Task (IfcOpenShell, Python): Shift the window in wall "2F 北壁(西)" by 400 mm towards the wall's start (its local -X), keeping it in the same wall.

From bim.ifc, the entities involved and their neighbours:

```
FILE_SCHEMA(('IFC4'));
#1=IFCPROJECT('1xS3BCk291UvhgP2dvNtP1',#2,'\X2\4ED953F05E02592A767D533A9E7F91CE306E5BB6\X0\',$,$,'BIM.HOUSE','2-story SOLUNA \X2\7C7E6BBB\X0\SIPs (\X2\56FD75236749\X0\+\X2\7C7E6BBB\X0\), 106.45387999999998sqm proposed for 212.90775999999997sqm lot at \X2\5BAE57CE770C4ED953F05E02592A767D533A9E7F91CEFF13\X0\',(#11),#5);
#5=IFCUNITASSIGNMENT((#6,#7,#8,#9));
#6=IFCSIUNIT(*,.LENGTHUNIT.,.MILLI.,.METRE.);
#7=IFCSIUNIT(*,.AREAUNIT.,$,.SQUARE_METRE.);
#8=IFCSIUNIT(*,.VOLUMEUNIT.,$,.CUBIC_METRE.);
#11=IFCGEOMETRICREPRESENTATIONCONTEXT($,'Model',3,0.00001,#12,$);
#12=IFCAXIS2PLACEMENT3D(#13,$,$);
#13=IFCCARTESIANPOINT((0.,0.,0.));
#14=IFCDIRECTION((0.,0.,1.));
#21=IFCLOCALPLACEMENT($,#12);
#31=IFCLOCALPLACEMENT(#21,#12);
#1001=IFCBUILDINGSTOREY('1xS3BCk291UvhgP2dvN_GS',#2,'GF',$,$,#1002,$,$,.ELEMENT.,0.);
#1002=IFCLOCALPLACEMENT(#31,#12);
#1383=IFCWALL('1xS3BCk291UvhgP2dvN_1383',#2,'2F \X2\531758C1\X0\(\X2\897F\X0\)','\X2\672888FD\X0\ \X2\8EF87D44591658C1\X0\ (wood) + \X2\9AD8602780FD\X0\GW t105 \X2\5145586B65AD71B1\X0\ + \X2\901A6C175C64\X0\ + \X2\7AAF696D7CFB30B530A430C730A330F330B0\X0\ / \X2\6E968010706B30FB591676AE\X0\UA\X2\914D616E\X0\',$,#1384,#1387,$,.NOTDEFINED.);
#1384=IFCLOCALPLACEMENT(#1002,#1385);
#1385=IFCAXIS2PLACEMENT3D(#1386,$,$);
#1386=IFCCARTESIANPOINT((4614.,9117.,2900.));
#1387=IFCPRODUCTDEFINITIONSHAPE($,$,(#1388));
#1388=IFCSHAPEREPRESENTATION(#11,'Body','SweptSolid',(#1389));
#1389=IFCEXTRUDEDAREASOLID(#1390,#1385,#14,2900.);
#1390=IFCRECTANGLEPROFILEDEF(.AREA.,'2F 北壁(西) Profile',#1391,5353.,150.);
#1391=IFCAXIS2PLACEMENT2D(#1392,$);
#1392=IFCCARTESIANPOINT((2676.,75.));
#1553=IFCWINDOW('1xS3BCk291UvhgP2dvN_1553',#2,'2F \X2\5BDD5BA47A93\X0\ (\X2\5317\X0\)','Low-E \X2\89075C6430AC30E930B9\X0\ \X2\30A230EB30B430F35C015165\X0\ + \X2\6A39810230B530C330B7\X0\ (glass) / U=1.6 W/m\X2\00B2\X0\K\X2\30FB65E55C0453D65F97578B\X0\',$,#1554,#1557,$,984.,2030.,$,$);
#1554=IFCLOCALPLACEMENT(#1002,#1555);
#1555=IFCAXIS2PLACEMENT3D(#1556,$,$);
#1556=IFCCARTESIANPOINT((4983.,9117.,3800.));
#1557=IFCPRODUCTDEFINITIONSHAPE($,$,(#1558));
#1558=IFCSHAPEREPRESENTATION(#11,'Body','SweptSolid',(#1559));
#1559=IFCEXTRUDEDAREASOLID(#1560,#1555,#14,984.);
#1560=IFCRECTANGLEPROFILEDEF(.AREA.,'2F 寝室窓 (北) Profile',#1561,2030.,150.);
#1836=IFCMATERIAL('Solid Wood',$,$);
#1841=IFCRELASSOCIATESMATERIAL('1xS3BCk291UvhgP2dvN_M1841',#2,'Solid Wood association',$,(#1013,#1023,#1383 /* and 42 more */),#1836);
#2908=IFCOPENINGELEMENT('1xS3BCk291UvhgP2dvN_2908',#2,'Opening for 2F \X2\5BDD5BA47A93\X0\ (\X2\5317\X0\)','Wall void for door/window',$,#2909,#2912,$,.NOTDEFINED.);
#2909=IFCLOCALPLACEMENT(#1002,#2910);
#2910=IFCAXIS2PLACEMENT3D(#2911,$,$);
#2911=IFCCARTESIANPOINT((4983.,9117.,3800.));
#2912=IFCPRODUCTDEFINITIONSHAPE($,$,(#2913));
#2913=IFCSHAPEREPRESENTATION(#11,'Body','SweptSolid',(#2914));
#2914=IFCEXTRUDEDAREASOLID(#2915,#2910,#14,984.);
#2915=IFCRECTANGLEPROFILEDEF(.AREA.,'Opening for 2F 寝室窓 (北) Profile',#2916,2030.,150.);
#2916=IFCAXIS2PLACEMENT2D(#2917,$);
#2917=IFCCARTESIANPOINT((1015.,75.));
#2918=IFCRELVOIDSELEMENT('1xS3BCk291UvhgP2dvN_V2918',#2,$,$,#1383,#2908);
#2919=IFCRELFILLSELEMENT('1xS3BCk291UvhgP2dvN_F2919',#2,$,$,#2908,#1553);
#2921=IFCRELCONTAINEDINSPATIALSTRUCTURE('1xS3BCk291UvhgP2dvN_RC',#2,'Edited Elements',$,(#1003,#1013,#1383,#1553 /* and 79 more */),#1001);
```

```python
import ifcopenshell
import ifcopenshell.api.geometry
import ifcopenshell.util.placement
import ifcopenshell.util.unit

model = ifcopenshell.open("bim.ifc")
unit_scale = ifcopenshell.util.unit.calculate_unit_scale(model)

window = model.by_guid("1xS3BCk291UvhgP2dvN_1553")
opening = window.FillsVoids[0].RelatingOpeningElement
wall = opening.VoidsElements[0].RelatingBuildingElement

wall_matrix = ifcopenshell.util.placement.get_local_placement(wall.ObjectPlacement)
shift = wall_matrix[:3, 0] * -0.4 / unit_scale
before = ifcopenshell.util.placement.get_local_placement(window.ObjectPlacement)[:3, 3].copy()

# The window is not placed relative to its opening, so move both.
for product in (opening, window):
    matrix = ifcopenshell.util.placement.get_local_placement(product.ObjectPlacement)
    matrix[:3, 3] += shift
    ifcopenshell.api.geometry.edit_object_placement(model, product=product, matrix=matrix, is_si=False)

after = ifcopenshell.util.placement.get_local_placement(window.ObjectPlacement)[:3, 3]
print("window moved by", (after - before).round(3) + 0.0)

model.write("bim_edited.ifc")
```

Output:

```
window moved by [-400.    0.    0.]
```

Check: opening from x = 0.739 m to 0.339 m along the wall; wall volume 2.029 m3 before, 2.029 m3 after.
